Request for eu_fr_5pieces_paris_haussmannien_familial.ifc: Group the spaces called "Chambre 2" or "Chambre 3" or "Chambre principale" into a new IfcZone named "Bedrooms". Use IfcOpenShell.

First a look at what the model holds.

```python
import ifcopenshell

model = ifcopenshell.open("eu_fr_5pieces_paris_haussmannien_familial.ifc")
print(model.schema)
seen = {}
for space in model.by_type("IfcSpace"):
    seen[space.LongName] = seen.get(space.LongName, 0) + 1
for name, count in sorted(seen.items(), key=str):
    print(count, "x", name)
print("zones:", [z.Name for z in model.by_type("IfcZone")][:20])
```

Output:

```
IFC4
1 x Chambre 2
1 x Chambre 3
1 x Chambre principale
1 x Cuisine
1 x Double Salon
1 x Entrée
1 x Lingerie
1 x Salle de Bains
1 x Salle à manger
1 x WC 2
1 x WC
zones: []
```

```python
import ifcopenshell
import ifcopenshell.api.group
import ifcopenshell.api.root

model = ifcopenshell.open("eu_fr_5pieces_paris_haussmannien_familial.ifc")

names = {"Chambre 2", "Chambre 3", "Chambre principale"}
spaces = [s for s in model.by_type("IfcSpace") if s.LongName in names]

zone = ifcopenshell.api.root.create_entity(model, ifc_class="IfcZone", name="Bedrooms")
ifcopenshell.api.group.assign_group(model, products=spaces, group=zone)
print(len(spaces), "spaces in", zone.Name)

model.write("eu_fr_5pieces_paris_haussmannien_familial_rev.ifc")
```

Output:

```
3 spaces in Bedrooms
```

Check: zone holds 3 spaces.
